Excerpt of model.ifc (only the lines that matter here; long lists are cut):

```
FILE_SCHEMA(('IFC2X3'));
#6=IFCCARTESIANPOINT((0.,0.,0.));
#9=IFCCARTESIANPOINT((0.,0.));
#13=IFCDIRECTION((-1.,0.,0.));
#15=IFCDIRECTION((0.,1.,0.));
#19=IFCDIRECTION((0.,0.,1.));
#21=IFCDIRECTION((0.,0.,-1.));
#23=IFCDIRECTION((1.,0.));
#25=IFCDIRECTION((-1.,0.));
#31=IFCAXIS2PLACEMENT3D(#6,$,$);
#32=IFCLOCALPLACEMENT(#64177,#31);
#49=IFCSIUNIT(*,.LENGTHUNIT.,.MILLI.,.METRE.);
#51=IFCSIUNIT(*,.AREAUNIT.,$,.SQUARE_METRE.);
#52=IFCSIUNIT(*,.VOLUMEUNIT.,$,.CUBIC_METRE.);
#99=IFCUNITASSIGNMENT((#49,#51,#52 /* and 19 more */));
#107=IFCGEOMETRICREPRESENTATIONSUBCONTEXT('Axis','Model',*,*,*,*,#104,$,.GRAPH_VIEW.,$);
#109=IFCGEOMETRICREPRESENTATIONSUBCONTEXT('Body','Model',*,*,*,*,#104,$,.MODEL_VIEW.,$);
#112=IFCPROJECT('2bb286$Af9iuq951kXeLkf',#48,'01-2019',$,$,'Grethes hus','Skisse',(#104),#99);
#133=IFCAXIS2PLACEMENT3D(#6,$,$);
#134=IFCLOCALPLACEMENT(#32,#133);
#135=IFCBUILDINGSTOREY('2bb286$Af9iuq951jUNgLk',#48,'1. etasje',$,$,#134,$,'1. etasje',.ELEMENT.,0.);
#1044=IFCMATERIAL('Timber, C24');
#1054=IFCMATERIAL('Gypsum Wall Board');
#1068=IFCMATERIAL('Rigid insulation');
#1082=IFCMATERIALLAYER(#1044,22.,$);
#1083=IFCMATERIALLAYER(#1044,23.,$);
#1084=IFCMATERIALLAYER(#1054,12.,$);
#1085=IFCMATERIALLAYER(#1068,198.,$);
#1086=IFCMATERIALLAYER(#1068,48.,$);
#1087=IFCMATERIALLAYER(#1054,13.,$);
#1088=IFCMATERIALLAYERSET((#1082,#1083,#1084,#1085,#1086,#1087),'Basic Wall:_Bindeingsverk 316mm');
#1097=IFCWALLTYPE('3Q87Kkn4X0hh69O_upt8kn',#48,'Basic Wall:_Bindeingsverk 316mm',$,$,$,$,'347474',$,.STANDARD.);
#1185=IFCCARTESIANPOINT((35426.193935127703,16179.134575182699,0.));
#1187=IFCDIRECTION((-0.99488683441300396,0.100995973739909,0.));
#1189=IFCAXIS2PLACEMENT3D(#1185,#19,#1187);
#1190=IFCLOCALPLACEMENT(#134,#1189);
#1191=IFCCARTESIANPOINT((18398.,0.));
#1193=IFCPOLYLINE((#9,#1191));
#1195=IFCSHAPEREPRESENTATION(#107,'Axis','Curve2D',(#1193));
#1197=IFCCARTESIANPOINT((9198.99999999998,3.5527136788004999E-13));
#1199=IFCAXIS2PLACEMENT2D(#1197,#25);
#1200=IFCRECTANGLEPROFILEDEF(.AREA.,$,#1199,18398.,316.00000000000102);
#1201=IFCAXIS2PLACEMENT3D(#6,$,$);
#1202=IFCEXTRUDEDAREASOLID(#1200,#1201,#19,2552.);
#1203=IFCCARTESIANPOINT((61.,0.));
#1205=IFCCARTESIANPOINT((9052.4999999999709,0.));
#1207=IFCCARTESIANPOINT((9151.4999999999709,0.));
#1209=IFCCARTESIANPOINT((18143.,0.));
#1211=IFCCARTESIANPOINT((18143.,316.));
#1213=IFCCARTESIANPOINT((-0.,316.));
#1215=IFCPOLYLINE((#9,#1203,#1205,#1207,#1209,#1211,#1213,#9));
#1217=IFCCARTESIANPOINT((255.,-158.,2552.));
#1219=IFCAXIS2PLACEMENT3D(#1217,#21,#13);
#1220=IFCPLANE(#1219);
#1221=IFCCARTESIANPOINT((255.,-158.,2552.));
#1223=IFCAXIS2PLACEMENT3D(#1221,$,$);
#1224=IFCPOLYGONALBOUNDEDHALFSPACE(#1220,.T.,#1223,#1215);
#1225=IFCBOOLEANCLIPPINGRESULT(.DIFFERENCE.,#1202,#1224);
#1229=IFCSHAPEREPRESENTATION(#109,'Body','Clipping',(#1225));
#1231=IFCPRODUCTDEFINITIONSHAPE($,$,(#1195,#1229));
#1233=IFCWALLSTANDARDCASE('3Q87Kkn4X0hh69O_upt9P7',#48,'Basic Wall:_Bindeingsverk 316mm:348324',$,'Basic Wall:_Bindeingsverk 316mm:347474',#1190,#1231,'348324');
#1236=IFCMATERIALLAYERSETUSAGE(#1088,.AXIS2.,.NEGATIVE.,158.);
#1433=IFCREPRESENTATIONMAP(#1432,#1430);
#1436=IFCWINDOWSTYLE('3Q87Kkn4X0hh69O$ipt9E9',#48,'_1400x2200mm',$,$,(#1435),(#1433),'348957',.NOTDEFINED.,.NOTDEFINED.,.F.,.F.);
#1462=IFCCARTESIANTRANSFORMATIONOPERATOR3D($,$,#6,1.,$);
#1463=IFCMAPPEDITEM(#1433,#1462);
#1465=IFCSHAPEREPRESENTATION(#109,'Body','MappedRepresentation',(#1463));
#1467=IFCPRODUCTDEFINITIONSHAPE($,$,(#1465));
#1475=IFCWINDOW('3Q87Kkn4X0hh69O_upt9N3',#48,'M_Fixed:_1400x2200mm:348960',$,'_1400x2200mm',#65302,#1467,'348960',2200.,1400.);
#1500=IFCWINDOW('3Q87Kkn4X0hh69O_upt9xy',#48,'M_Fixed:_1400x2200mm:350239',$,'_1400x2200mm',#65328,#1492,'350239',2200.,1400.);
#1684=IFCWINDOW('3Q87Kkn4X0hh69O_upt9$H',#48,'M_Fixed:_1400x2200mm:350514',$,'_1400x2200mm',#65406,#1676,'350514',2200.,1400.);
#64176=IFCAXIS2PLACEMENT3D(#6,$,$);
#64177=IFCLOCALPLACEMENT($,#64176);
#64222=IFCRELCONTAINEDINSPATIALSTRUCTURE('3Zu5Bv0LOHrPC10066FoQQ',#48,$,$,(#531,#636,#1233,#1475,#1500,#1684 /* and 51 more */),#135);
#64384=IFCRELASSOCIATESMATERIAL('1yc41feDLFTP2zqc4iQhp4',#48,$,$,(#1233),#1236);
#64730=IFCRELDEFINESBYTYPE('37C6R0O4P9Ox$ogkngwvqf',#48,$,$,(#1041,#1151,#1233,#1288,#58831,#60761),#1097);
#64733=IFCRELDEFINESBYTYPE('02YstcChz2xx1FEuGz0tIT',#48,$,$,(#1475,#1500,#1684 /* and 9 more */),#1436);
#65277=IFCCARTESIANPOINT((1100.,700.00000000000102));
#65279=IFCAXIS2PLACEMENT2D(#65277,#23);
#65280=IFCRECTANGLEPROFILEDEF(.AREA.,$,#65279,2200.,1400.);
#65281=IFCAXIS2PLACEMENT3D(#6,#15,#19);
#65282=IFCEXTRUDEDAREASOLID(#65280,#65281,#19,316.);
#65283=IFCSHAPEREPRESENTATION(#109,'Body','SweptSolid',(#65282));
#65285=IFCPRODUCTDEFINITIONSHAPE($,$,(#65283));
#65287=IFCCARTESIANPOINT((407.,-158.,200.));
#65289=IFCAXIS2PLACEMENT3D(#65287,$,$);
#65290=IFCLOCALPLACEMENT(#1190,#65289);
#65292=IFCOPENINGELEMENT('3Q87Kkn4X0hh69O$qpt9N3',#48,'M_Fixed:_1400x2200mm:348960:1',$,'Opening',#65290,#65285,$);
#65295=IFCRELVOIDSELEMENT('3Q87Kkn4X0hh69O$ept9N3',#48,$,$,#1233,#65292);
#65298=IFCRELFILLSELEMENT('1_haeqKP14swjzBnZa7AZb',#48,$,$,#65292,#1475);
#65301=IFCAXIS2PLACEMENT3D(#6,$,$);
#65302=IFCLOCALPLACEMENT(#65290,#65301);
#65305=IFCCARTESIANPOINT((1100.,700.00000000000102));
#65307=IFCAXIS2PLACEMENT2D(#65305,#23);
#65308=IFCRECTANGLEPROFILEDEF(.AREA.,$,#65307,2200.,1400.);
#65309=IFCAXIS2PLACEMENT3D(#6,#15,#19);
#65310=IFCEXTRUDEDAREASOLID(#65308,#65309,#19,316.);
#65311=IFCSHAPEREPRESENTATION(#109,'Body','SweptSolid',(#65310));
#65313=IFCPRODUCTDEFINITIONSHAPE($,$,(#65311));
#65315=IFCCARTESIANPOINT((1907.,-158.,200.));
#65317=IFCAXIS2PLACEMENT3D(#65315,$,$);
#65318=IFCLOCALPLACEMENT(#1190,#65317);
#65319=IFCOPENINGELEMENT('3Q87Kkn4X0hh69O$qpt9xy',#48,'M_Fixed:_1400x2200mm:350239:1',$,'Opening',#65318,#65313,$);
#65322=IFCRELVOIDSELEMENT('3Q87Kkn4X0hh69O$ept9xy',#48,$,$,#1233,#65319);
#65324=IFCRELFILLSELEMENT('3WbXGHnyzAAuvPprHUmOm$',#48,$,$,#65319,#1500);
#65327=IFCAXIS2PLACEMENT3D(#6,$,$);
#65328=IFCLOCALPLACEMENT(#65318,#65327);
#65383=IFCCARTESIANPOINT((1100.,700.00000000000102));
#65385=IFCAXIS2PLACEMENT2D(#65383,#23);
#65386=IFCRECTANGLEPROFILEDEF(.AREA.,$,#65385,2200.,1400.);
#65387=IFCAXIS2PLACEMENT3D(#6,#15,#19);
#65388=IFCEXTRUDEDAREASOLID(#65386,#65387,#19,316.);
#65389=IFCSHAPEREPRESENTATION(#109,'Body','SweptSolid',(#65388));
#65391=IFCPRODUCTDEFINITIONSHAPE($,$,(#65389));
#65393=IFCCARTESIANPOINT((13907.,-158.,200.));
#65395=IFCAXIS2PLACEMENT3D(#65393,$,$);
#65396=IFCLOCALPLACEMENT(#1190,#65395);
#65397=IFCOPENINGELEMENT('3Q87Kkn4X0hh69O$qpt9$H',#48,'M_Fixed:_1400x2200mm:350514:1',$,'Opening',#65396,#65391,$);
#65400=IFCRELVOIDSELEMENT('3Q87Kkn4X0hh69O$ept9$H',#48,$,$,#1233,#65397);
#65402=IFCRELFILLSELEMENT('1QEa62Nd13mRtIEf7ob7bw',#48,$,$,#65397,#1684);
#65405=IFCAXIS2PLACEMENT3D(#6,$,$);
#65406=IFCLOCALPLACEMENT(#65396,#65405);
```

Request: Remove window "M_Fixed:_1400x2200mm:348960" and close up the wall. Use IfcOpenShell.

```python
import ifcopenshell
import ifcopenshell.api.feature
import ifcopenshell.api.root
import ifcopenshell.geom
import ifcopenshell.util.shape

model = ifcopenshell.open("model.ifc")
settings = ifcopenshell.geom.settings()


def volume(element):
    """Net volume in cubic metres, openings subtracted."""
    shape = ifcopenshell.geom.create_shape(settings, element)
    return ifcopenshell.util.shape.get_volume(shape.geometry)


window = model.by_guid("3Q87Kkn4X0hh69O_upt9N3")
opening = window.FillsVoids[0].RelatingOpeningElement
wall = opening.VoidsElements[0].RelatingBuildingElement
before = volume(wall)

ifcopenshell.api.root.remove_product(model, product=window)
ifcopenshell.api.feature.remove_feature(model, feature=opening)

after = volume(wall)

print(f"wall volume {before:.3f} -> {after:.3f} m3")

model.write("model-out.ifc")
```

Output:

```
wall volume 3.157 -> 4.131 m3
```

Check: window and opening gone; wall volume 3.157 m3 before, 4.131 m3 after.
